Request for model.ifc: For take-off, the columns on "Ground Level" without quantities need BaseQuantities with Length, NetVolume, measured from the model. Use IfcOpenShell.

First a look at what the model holds.

```python
import ifcopenshell
import ifcopenshell.util.element
import ifcopenshell.util.unit

model = ifcopenshell.open("model.ifc")
print(model.schema)
for unit_type in ("LENGTHUNIT", "AREAUNIT", "VOLUMEUNIT"):
    print(unit_type, ifcopenshell.util.unit.calculate_unit_scale(model, unit_type))
storey = next(s for s in model.by_type("IfcBuildingStorey") if s.Name == "Ground Level")
columns = [e for e in ifcopenshell.util.element.get_decomposition(storey) if e.is_a("IfcColumn")]
for e in sorted(columns, key=lambda e: e.id()):
    print(e.id(), e.is_a(), e.Name, list(ifcopenshell.util.element.get_psets(e, qtos_only=True)), sep=" | ")
```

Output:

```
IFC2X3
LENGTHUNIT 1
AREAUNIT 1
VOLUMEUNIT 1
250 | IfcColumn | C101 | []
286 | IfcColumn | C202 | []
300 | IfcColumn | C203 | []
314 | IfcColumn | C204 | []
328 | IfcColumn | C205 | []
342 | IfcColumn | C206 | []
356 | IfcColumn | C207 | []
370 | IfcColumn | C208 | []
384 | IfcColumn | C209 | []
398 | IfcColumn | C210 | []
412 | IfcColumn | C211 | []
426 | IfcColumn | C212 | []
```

```python
import ifcopenshell
import ifcopenshell.api.pset
import ifcopenshell.geom
import ifcopenshell.util.element
import ifcopenshell.util.shape
import ifcopenshell.util.unit

model = ifcopenshell.open("model.ifc")
unit_scale = ifcopenshell.util.unit.calculate_unit_scale(model)
volume_scale = ifcopenshell.util.unit.calculate_unit_scale(model, "VOLUMEUNIT")
settings = ifcopenshell.geom.settings()

storey = next(s for s in model.by_type("IfcBuildingStorey") if s.Name == "Ground Level")
columns = [e for e in ifcopenshell.util.element.get_decomposition(storey) if e.is_a("IfcColumn")]

for e in sorted(columns, key=lambda e: e.id()):
    if ifcopenshell.util.element.get_psets(e, qtos_only=True, should_inherit=False):
        continue
    # Geometry comes back in metres, in the element's own axes.
    shape = ifcopenshell.geom.create_shape(settings, e)
    values = {
        "Length": ifcopenshell.util.shape.get_z(shape.geometry) / unit_scale,
        "NetVolume": ifcopenshell.util.shape.get_volume(shape.geometry) / volume_scale,
    }
    qto = ifcopenshell.api.pset.add_qto(model, product=e, name="BaseQuantities")
    ifcopenshell.api.pset.edit_qto(model, qto=qto, properties=values)
    print(e.id(), {k: round(v, 3) for k, v in values.items()})

model.write("model_v2.ifc")
```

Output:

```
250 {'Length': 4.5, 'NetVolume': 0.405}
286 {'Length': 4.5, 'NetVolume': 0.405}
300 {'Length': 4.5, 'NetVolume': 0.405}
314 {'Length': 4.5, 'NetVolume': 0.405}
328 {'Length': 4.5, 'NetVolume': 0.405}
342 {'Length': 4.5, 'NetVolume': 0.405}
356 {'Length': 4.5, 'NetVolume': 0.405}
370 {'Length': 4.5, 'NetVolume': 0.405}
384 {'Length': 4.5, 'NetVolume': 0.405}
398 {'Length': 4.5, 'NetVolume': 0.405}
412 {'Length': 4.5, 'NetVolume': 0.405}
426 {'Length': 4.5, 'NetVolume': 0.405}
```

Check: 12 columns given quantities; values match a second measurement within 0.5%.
